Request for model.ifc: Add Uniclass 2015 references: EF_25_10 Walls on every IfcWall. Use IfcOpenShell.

First a look at what the model holds.

```python
import ifcopenshell

model = ifcopenshell.open("model.ifc")
print(model.schema)
print("classifications:", [c.Name for c in model.by_type("IfcClassification")])
for ifc_class in ("IfcDoor", "IfcRoof", "IfcStair", "IfcWall", "IfcWindow"):
    print(ifc_class, len(model.by_type(ifc_class)))
```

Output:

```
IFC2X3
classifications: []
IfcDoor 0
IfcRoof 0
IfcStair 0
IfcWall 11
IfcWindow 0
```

```python
import ifcopenshell
import ifcopenshell.api.classification

model = ifcopenshell.open("model.ifc")

# IFC2X3 requires Source and Edition and has no link from the project to the system.
system = model.create_entity("IfcClassification", Source="NBS", Edition="2015", Name="Uniclass 2015")

codes = {
    "IfcWall": ("EF_25_10", "Walls"),
}
for ifc_class, (code, name) in codes.items():
    products = model.by_type(ifc_class)
    ifcopenshell.api.classification.add_reference(
        model, products=products, classification=system, identification=code, name=name
    )
    print(code, len(products))

model.write("model_rev.ifc")
```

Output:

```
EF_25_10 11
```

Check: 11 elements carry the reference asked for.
